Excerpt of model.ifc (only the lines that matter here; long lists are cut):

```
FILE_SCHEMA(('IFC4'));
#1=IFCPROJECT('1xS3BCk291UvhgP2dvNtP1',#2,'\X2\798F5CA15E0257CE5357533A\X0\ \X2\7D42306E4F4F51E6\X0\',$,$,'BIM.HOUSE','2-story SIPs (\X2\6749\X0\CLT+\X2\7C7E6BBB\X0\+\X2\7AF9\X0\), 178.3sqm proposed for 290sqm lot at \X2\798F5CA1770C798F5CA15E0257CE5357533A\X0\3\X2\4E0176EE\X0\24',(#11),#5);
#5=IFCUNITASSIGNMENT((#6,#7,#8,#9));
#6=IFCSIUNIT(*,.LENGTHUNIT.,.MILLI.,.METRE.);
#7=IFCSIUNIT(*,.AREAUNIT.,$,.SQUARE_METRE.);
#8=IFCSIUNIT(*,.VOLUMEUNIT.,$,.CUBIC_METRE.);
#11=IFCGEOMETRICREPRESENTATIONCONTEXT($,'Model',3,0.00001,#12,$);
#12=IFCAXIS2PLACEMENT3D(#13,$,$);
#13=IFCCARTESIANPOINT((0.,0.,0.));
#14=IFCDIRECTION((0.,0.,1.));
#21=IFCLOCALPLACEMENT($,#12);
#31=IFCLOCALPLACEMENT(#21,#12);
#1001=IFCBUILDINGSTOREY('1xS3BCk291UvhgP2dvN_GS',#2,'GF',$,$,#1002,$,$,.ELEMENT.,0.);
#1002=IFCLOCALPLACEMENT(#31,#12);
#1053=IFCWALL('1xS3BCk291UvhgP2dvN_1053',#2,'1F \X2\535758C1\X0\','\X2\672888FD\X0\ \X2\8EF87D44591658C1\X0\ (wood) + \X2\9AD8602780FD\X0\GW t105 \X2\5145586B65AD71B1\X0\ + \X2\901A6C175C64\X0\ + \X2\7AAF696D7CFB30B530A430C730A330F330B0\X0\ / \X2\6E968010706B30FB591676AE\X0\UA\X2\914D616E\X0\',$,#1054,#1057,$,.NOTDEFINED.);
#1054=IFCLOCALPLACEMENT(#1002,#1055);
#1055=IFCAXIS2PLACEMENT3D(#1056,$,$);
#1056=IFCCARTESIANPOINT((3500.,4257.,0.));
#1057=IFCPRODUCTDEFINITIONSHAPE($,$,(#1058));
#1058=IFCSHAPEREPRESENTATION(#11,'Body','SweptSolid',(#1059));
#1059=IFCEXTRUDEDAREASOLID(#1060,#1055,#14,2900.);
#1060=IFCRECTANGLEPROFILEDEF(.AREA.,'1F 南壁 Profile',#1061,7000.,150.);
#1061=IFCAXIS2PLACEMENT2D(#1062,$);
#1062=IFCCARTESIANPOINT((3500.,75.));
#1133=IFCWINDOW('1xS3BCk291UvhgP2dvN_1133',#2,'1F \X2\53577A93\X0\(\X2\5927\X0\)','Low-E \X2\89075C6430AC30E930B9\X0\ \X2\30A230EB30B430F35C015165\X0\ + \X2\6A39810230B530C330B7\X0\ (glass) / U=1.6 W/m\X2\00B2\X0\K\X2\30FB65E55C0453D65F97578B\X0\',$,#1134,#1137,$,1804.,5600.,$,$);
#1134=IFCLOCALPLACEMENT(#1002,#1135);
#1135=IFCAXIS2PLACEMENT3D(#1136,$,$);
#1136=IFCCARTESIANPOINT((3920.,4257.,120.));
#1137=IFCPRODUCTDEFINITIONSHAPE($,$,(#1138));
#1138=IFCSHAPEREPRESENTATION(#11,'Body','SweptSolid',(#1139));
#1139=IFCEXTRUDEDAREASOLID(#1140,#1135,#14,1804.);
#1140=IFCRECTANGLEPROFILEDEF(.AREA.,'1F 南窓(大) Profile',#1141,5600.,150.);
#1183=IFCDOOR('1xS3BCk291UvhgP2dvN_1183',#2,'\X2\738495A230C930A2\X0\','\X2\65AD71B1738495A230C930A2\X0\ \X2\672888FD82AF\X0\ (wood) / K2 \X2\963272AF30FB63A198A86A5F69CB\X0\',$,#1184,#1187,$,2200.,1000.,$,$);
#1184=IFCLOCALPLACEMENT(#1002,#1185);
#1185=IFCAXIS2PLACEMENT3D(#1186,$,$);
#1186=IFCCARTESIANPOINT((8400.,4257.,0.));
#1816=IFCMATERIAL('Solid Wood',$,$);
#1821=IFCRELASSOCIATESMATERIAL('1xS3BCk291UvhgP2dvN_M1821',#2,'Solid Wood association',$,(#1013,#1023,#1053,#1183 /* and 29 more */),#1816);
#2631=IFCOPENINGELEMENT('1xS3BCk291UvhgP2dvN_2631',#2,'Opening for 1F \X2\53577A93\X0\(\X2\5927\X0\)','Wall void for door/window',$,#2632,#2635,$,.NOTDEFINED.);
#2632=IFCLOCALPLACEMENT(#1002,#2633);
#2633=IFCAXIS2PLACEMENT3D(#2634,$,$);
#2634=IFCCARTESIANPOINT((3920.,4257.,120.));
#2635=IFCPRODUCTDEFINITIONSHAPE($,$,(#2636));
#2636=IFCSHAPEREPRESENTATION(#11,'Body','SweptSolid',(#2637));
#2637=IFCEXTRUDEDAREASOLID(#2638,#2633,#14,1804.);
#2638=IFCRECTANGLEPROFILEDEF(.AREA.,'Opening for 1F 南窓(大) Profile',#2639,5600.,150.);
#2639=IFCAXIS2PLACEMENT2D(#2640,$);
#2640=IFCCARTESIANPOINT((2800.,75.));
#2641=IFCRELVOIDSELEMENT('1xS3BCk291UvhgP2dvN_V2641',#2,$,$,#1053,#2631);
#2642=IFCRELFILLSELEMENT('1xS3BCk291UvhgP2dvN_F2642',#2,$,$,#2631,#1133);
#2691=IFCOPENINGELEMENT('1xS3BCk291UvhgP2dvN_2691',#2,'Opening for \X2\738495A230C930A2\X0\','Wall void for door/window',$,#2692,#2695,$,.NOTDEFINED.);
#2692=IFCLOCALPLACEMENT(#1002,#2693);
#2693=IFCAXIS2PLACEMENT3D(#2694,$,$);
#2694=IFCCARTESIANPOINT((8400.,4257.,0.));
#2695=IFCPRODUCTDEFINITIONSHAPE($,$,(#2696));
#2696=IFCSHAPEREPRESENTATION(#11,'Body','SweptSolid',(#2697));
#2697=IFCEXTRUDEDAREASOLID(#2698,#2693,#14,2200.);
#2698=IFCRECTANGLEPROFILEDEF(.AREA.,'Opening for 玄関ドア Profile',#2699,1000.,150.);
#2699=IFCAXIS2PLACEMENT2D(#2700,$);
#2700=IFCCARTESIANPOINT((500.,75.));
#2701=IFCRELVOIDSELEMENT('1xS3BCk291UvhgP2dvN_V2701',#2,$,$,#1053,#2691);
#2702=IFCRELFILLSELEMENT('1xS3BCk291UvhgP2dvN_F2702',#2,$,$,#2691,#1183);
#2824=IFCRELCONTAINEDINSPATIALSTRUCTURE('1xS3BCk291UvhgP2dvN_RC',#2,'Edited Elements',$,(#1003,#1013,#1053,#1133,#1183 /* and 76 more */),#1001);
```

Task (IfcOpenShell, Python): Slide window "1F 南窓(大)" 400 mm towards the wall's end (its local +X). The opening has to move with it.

```python
import ifcopenshell
import ifcopenshell.api.geometry
import ifcopenshell.util.placement
import ifcopenshell.util.unit

model = ifcopenshell.open("model.ifc")
unit_scale = ifcopenshell.util.unit.calculate_unit_scale(model)

window = model.by_guid("1xS3BCk291UvhgP2dvN_1133")
opening = window.FillsVoids[0].RelatingOpeningElement
wall = opening.VoidsElements[0].RelatingBuildingElement

wall_matrix = ifcopenshell.util.placement.get_local_placement(wall.ObjectPlacement)
shift = wall_matrix[:3, 0] * 0.4 / unit_scale
before = ifcopenshell.util.placement.get_local_placement(window.ObjectPlacement)[:3, 3].copy()

# The window is not placed relative to its opening, so move both.
for product in (opening, window):
    matrix = ifcopenshell.util.placement.get_local_placement(product.ObjectPlacement)
    matrix[:3, 3] += shift
    ifcopenshell.api.geometry.edit_object_placement(model, product=product, matrix=matrix, is_si=False)

after = ifcopenshell.util.placement.get_local_placement(window.ObjectPlacement)[:3, 3]
print("window moved by", (after - before).round(3) + 0.0)

model.write("model_updated.ifc")
```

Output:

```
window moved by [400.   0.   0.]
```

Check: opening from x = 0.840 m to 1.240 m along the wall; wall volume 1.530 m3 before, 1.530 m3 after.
